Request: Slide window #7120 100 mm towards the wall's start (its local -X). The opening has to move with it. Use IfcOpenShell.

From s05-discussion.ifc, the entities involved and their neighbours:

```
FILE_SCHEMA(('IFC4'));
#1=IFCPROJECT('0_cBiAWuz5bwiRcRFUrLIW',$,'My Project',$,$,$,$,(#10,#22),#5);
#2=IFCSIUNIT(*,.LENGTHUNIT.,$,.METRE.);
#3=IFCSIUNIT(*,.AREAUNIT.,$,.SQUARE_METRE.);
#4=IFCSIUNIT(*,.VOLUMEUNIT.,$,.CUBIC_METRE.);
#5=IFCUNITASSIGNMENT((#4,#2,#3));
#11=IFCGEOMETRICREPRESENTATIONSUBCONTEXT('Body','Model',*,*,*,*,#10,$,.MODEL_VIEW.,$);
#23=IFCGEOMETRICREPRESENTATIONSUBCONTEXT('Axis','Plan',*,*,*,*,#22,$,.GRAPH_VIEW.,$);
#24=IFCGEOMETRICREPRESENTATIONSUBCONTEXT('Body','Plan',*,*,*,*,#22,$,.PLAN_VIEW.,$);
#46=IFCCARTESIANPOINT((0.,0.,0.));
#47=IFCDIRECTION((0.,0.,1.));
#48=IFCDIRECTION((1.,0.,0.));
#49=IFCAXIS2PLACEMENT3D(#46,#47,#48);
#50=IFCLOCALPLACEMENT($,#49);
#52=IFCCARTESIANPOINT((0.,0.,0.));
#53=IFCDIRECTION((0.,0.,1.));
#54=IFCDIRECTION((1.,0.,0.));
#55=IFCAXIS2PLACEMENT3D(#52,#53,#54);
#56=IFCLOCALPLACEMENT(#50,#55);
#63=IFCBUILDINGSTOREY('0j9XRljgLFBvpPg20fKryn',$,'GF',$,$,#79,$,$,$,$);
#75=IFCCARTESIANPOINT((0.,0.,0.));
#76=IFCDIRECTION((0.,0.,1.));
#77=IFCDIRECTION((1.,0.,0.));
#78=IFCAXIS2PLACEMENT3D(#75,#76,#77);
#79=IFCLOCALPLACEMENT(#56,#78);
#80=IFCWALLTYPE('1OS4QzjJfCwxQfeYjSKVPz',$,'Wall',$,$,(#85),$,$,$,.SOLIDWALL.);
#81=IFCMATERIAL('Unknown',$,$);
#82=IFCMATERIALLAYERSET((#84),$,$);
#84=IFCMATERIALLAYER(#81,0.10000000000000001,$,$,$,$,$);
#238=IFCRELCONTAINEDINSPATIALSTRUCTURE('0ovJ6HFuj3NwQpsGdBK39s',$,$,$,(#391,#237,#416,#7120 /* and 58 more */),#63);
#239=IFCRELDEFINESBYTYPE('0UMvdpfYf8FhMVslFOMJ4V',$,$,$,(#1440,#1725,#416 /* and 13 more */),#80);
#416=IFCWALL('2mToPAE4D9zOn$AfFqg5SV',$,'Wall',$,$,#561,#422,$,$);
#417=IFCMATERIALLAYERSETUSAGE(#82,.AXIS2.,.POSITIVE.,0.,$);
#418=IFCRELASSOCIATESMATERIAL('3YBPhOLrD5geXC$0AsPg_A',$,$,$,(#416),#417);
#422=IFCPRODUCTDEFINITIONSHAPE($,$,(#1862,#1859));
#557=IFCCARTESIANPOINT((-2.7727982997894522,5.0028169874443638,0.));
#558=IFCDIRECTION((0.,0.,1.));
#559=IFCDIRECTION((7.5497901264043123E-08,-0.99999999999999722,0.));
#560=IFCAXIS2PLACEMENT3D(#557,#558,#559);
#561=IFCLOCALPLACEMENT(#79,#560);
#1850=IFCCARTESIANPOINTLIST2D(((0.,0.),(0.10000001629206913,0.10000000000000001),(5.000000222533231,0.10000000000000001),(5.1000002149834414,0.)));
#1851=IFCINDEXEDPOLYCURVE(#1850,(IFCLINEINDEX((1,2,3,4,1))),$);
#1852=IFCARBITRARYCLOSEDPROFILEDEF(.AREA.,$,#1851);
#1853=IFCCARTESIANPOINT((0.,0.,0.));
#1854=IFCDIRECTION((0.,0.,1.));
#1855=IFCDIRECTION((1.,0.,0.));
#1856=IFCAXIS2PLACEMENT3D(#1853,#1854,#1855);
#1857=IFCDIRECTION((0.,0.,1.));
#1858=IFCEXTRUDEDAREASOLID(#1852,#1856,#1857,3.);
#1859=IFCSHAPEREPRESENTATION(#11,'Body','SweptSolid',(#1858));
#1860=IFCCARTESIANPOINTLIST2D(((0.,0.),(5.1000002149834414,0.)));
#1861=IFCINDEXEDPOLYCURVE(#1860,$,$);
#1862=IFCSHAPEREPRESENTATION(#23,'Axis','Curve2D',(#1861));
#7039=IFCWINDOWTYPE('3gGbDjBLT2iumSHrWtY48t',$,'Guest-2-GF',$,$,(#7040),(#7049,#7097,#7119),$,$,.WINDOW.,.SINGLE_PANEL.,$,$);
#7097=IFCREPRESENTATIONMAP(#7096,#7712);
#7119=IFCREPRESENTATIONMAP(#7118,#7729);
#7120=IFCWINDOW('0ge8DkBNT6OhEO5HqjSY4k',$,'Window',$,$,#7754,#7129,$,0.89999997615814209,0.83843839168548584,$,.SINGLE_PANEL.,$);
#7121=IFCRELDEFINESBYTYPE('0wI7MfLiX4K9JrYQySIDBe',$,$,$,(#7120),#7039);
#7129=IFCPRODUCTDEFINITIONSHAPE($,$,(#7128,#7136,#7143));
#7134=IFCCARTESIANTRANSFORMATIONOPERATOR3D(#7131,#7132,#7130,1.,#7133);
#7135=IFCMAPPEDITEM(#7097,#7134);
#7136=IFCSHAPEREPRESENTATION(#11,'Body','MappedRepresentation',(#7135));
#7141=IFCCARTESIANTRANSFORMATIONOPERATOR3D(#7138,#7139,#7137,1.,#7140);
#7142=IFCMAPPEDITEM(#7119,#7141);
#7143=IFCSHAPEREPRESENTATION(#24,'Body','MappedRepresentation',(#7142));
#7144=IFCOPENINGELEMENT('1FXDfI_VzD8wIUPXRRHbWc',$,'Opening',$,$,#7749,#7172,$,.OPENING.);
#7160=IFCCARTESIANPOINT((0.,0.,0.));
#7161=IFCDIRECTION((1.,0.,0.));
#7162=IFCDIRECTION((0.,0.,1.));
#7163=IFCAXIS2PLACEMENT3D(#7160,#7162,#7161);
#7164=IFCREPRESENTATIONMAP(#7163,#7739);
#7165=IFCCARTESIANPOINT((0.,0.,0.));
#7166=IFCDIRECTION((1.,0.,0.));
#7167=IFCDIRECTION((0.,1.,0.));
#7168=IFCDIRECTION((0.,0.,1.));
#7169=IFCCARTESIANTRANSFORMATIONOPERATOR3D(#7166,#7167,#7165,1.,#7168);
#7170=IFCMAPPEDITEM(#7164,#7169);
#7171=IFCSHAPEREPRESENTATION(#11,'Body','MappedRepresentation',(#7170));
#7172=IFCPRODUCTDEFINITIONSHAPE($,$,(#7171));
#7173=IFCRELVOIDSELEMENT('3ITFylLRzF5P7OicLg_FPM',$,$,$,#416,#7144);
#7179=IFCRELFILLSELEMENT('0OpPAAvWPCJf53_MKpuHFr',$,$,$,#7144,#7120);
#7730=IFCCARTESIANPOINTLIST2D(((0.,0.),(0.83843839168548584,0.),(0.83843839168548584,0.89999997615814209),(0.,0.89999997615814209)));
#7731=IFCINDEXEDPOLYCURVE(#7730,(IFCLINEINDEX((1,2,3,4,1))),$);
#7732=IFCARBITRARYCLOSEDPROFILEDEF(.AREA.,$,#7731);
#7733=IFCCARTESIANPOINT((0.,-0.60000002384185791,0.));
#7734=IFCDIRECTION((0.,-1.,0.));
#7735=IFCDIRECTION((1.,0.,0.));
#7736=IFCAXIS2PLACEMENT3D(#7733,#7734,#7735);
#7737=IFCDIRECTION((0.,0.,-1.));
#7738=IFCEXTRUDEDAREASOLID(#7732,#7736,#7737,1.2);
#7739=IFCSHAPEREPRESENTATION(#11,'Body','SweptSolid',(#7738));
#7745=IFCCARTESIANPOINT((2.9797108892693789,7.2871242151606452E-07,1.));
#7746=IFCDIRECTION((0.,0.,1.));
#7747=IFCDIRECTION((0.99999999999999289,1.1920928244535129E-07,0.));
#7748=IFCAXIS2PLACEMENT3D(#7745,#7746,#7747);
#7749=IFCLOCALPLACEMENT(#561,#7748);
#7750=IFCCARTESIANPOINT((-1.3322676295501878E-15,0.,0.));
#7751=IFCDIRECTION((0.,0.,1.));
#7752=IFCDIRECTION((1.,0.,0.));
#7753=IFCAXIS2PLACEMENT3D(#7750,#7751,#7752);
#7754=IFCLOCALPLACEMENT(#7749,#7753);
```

```python
import ifcopenshell
import ifcopenshell.api.geometry
import ifcopenshell.util.placement
import ifcopenshell.util.unit

model = ifcopenshell.open("s05-discussion.ifc")
unit_scale = ifcopenshell.util.unit.calculate_unit_scale(model)

window = model.by_guid("0ge8DkBNT6OhEO5HqjSY4k")
opening = window.FillsVoids[0].RelatingOpeningElement
wall = opening.VoidsElements[0].RelatingBuildingElement

wall_matrix = ifcopenshell.util.placement.get_local_placement(wall.ObjectPlacement)
shift = wall_matrix[:3, 0] * -0.1 / unit_scale
before = ifcopenshell.util.placement.get_local_placement(window.ObjectPlacement)[:3, 3].copy()

# The window is placed relative to its opening, so it follows when the opening moves.
matrix = ifcopenshell.util.placement.get_local_placement(opening.ObjectPlacement)
matrix[:3, 3] += shift
ifcopenshell.api.geometry.edit_object_placement(
    model, product=opening, matrix=matrix, is_si=False, should_transform_children=True
)

after = ifcopenshell.util.placement.get_local_placement(window.ObjectPlacement)[:3, 3]
print("window moved by", (after - before).round(3) + 0.0)

model.write("s05-discussion_rev.ifc")
```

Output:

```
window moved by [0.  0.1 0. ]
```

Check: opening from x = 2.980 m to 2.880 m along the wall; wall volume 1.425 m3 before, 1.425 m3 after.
